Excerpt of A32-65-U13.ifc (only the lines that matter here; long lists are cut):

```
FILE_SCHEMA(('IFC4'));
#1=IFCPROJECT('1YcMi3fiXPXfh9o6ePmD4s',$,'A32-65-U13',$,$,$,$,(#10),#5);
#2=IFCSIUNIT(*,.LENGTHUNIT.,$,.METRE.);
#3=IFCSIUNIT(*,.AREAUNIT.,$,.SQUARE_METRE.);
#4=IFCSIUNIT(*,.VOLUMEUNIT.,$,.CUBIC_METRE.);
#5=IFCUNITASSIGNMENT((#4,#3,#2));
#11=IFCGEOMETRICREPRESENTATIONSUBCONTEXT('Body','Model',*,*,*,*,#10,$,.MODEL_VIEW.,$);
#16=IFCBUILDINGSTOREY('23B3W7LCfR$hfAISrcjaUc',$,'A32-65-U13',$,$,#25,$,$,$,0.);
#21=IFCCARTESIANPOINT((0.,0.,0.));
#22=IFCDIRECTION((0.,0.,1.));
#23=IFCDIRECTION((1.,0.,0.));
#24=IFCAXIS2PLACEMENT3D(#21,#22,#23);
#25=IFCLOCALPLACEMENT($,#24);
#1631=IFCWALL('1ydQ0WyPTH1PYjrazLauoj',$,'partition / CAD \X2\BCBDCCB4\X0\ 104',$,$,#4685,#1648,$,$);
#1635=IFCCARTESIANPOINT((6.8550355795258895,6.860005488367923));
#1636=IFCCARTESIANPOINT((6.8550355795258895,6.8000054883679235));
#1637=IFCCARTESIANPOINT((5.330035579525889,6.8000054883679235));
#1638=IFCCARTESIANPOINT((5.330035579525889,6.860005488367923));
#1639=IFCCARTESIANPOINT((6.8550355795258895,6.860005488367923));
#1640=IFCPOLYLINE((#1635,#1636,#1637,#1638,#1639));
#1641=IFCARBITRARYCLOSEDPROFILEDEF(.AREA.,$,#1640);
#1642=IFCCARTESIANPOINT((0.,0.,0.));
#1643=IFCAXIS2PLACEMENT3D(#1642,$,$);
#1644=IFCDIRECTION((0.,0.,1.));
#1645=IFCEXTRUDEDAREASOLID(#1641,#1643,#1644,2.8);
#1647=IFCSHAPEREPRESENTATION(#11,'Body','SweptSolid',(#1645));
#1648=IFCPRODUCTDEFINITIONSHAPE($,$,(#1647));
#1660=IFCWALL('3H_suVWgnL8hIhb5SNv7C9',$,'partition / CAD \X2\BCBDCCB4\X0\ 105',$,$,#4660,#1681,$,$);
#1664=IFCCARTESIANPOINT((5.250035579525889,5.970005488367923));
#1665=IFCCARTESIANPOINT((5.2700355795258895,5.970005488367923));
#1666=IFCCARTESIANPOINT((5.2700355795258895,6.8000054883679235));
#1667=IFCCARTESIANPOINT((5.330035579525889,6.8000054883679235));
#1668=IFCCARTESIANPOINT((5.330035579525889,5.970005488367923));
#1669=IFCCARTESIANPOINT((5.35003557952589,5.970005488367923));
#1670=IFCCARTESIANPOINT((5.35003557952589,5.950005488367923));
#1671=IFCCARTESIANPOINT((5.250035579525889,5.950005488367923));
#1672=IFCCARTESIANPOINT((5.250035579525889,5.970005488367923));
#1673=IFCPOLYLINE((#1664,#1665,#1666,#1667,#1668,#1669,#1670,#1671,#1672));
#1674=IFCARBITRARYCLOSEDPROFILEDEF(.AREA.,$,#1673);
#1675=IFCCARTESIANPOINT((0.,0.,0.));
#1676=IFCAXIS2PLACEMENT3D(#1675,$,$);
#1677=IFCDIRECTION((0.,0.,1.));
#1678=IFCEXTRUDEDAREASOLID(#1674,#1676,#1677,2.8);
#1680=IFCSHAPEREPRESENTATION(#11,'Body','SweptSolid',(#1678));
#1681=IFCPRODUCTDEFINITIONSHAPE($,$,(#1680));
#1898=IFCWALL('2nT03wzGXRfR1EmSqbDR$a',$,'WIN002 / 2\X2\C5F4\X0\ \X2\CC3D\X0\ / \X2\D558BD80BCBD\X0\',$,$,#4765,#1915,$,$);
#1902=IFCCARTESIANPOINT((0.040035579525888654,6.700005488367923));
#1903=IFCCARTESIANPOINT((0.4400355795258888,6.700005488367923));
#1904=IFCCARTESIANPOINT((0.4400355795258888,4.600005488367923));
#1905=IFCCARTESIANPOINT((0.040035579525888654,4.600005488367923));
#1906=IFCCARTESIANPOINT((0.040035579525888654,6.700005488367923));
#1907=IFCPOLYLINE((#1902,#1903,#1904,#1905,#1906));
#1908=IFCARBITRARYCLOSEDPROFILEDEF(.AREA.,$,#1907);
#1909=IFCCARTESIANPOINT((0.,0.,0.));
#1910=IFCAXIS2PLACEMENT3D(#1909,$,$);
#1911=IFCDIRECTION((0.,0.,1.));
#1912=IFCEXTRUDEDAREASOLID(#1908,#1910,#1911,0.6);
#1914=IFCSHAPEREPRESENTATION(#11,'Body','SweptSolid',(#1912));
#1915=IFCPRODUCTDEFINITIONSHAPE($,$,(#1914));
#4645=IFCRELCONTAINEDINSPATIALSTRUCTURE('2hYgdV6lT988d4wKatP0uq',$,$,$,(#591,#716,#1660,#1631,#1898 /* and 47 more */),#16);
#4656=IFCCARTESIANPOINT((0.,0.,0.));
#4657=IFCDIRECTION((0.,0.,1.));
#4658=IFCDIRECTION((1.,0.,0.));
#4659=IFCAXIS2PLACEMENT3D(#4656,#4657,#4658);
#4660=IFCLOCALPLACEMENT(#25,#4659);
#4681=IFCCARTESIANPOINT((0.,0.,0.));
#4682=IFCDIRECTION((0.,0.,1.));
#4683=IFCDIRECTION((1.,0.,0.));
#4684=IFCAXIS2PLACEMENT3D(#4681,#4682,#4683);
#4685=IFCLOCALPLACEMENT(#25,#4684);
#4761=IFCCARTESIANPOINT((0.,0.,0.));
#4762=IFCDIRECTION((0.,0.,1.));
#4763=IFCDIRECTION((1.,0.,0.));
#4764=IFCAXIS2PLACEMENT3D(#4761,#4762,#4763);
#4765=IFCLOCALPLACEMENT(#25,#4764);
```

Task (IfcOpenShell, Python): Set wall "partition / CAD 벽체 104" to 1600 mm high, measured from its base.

```python
import ifcopenshell
import ifcopenshell.geom
import ifcopenshell.util.representation
import ifcopenshell.util.shape
import ifcopenshell.util.unit

model = ifcopenshell.open("A32-65-U13.ifc")
unit_scale = ifcopenshell.util.unit.calculate_unit_scale(model)
settings = ifcopenshell.geom.settings()


def volume(element):
    """Net volume in cubic metres, openings subtracted."""
    shape = ifcopenshell.geom.create_shape(settings, element)
    return ifcopenshell.util.shape.get_volume(shape.geometry)


wall = model.by_guid("1ydQ0WyPTH1PYjrazLauoj")
before = volume(wall)

body = ifcopenshell.util.representation.get_representation(wall, "Model", "Body")
solid = body.Items[0]
old_height = solid.Depth
solid.Depth = 1.6 / unit_scale
after = volume(wall)

print(f"height {old_height:g} -> {solid.Depth:g}, volume {before:.3f} -> {after:.3f} m3")

model.write("A32-65-U13-out.ifc")
```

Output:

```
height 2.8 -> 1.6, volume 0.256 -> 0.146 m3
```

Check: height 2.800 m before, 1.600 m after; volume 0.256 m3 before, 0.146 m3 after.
